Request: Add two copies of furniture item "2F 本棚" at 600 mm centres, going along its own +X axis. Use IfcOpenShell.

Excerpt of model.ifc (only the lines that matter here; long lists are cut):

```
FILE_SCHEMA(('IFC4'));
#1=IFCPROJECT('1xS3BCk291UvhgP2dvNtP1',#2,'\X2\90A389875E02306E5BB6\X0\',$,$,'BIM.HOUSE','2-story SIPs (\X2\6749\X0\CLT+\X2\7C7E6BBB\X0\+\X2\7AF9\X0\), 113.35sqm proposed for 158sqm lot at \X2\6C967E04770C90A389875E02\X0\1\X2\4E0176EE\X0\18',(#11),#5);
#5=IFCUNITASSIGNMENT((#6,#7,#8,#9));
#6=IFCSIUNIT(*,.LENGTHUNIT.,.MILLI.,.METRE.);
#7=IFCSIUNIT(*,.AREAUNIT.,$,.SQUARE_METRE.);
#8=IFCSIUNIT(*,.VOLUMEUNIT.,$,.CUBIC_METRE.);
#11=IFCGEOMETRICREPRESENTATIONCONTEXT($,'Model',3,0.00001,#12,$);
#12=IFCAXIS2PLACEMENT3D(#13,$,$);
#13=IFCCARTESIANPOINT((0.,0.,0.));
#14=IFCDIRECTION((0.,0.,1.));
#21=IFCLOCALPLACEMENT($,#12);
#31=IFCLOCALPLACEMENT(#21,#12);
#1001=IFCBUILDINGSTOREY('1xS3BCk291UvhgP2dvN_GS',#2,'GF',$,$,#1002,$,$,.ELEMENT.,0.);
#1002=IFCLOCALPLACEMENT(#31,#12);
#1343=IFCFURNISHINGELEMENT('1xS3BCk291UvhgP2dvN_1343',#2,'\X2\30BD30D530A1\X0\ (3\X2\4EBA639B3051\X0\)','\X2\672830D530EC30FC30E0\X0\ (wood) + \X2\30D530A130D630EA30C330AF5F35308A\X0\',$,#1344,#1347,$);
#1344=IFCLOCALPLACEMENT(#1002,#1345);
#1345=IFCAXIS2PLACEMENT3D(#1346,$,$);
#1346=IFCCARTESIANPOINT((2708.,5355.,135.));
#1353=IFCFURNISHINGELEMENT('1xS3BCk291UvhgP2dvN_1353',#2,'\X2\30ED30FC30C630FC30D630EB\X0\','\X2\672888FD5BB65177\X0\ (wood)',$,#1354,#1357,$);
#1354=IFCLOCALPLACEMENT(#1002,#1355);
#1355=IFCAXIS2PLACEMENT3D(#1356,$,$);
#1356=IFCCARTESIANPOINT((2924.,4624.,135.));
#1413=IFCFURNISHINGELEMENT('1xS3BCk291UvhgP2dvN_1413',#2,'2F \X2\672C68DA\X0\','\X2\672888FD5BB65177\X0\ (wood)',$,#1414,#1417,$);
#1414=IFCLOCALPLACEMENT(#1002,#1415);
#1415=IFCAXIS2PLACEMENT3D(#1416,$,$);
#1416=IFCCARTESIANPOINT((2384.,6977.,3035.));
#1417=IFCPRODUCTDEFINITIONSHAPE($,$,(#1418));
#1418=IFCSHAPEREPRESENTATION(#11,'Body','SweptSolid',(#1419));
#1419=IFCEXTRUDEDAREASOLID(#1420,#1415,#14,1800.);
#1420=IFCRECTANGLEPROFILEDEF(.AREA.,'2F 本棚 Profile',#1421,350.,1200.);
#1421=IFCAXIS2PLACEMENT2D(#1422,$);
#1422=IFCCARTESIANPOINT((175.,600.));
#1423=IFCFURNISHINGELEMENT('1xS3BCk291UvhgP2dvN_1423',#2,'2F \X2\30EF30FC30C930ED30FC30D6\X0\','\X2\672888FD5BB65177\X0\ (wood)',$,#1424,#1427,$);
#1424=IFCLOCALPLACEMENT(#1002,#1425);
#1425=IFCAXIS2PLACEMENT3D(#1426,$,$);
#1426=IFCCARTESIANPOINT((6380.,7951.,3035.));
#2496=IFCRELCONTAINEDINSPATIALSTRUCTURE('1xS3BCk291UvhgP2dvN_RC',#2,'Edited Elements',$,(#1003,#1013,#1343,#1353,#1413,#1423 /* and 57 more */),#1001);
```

```python
import ifcopenshell
import ifcopenshell.api.geometry
import ifcopenshell.api.root
import ifcopenshell.util.element
import ifcopenshell.util.placement

model = ifcopenshell.open("model.ifc")


def reuse_history(source, copy):
    """copy_class also copies each property set's owner history, people and application; keep the originals."""
    for rel in copy.IsDefinedBy:
        if rel.is_a("IfcRelDefinesByProperties") and (history := rel.RelatingPropertyDefinition.OwnerHistory):
            rel.RelatingPropertyDefinition.OwnerHistory = source.OwnerHistory
            ifcopenshell.util.element.remove_deep2(model, history)


source = model.by_guid("1xS3BCk291UvhgP2dvN_1413")
base = ifcopenshell.util.placement.get_local_placement(source.ObjectPlacement)
step = base[:3, 0] * 600.0

for i in range(1, 3):
    copy = ifcopenshell.api.root.copy_class(model, product=source)
    copy.Representation = ifcopenshell.util.element.copy_deep(
        model, source.Representation, exclude=["IfcGeometricRepresentationContext", "IfcRepresentationMap"]
    )
    reuse_history(source, copy)
    matrix = base.copy()
    matrix[:3, 3] += i * step
    print("added at", matrix[:3, 3].round(3) + 0.0)
    ifcopenshell.api.geometry.edit_object_placement(model, product=copy, matrix=matrix, is_si=False)

model.write("model_v2.ifc")
```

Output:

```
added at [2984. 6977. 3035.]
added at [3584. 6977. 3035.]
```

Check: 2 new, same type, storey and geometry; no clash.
